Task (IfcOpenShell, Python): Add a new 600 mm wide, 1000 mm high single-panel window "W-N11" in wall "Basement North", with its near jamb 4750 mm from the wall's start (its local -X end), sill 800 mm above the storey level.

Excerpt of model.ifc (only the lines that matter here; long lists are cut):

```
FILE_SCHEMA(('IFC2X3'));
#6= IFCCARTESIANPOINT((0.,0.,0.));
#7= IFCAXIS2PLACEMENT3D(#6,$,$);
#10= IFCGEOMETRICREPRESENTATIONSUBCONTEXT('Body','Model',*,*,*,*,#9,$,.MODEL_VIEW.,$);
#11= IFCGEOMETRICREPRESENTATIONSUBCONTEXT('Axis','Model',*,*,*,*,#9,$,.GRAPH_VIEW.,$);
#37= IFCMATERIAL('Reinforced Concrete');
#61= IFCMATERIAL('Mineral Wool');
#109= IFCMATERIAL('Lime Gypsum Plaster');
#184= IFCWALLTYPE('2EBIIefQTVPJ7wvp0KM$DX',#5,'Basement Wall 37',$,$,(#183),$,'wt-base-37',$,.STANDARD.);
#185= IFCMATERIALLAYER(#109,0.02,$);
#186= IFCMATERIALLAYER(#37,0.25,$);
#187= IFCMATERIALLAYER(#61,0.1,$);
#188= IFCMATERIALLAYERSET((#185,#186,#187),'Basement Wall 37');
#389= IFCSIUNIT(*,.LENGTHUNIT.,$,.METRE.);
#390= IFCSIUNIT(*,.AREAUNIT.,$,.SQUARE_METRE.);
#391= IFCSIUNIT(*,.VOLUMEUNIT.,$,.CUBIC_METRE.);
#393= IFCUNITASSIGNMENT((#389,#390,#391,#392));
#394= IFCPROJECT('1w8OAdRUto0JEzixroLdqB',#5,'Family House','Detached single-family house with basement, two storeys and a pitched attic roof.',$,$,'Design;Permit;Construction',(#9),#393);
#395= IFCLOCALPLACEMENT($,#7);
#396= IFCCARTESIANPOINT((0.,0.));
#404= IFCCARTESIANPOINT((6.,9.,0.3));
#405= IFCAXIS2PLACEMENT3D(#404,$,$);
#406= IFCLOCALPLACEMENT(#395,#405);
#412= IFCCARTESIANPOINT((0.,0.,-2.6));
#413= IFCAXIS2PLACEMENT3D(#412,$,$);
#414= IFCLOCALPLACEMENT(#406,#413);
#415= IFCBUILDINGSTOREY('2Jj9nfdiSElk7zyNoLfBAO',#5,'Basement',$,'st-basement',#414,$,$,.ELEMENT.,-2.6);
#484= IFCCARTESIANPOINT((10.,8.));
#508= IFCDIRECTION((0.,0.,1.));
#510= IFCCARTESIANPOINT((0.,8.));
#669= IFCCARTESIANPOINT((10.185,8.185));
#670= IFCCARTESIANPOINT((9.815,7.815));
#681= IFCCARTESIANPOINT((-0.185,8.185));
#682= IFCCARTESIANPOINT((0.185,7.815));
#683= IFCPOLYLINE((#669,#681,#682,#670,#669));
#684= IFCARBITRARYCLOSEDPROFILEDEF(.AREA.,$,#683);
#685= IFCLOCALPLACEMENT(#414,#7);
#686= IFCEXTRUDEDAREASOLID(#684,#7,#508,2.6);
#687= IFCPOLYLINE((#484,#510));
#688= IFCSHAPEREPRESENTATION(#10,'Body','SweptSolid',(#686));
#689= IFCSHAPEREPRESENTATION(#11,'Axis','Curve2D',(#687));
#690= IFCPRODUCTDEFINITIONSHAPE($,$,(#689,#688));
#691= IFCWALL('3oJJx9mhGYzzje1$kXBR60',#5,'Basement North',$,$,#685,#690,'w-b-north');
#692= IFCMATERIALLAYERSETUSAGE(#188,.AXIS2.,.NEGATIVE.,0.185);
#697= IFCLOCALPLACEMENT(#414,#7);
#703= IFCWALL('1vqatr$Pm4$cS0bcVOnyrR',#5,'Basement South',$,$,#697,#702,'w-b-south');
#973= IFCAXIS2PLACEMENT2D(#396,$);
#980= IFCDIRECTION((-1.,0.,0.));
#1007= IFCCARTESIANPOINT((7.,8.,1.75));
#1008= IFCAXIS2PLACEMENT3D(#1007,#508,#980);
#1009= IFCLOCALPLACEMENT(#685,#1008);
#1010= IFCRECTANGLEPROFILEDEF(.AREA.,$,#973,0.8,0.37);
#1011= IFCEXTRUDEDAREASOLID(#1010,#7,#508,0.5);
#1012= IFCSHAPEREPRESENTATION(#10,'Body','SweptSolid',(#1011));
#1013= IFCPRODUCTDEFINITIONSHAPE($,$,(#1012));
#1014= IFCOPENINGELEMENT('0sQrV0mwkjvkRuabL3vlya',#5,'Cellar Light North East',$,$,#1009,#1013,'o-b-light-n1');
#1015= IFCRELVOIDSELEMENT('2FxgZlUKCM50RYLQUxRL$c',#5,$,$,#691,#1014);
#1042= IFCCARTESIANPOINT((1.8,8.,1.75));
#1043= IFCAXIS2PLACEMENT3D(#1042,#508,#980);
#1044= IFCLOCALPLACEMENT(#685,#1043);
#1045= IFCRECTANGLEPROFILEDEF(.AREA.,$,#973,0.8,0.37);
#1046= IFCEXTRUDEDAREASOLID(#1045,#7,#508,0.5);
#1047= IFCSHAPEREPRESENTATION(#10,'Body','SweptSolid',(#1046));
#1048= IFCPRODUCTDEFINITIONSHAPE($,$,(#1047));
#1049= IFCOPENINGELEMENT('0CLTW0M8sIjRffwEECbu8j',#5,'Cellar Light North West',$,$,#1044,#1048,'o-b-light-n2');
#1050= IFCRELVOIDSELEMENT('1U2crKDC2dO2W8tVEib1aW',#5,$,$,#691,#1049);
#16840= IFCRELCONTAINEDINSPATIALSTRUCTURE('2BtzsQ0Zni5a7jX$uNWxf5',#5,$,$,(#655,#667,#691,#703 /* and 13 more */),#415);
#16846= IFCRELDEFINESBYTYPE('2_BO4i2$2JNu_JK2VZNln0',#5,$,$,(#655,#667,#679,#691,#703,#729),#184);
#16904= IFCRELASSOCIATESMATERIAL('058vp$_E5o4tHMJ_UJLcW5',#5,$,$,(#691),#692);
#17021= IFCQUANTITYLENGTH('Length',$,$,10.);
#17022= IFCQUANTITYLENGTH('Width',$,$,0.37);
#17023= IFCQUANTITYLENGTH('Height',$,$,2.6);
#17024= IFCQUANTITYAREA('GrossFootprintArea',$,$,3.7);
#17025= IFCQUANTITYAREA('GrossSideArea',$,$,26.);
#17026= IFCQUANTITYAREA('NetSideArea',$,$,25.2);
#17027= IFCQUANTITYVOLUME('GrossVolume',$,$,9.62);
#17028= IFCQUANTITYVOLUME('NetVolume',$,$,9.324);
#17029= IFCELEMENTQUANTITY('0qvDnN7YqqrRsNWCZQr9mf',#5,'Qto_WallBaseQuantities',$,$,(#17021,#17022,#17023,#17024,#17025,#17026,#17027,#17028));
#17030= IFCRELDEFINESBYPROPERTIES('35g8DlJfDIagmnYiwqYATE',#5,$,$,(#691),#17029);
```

```python
import numpy as np
import ifcopenshell
import ifcopenshell.api.feature
import ifcopenshell.api.geometry
import ifcopenshell.api.pset
import ifcopenshell.api.root
import ifcopenshell.api.spatial
import ifcopenshell.api.type
import ifcopenshell.geom
import ifcopenshell.util.element
import ifcopenshell.util.placement
import ifcopenshell.util.representation
import ifcopenshell.util.shape
import ifcopenshell.util.unit

model = ifcopenshell.open("model.ifc")
unit_scale = ifcopenshell.util.unit.calculate_unit_scale(model)
area_scale = ifcopenshell.util.unit.calculate_unit_scale(model, "AREAUNIT")
volume_scale = ifcopenshell.util.unit.calculate_unit_scale(model, "VOLUMEUNIT")
settings = ifcopenshell.geom.settings()


def volume(element):
    """Net volume in cubic metres, openings subtracted."""
    shape = ifcopenshell.geom.create_shape(settings, element)
    return ifcopenshell.util.shape.get_volume(shape.geometry)


wall = model.by_guid("3oJJx9mhGYzzje1$kXBR60")
storey = ifcopenshell.util.element.get_container(wall, ifc_class="IfcBuildingStorey")
context = ifcopenshell.util.representation.get_context(model, "Model", "Body", "MODEL_VIEW")
before = volume(wall)

width, height, from_end, sill = 0.6, 1, 4.75, 0.8  # metres

# The wall runs along its own X axis, and the end named is its -X end.
wall_shape = ifcopenshell.geom.create_shape(settings, wall)
x, y, z = ifcopenshell.util.shape.get_vertices(wall_shape.geometry).T
start = x.min() + from_end
face, thickness = float(y.min()), float(y.max() - y.min())
wall_matrix = ifcopenshell.util.placement.get_local_placement(wall.ObjectPlacement)
level = ifcopenshell.util.placement.get_local_placement(storey.ObjectPlacement)[2, 3]


def in_wall(x, y):
    """Placement at x, y metres in the wall's axes, at sill height."""
    matrix = wall_matrix.copy()
    matrix[:, 3] = wall_matrix @ np.array([x / unit_scale, y / unit_scale, 0.0, 1.0])
    matrix[2, 3] = level + sill / unit_scale
    return matrix


# Opening: a box that overshoots both wall faces by 50 mm.
opening = ifcopenshell.api.root.create_entity(model, ifc_class="IfcOpeningElement")
box = ifcopenshell.api.geometry.add_wall_representation(
    model, context=context, length=width, height=height, thickness=thickness + 0.1
)
ifcopenshell.api.geometry.assign_representation(model, product=opening, representation=box)
ifcopenshell.api.geometry.edit_object_placement(model, product=opening, matrix=in_wall(start, face - 0.05), is_si=False)
ifcopenshell.api.feature.add_feature(model, feature=opening, element=wall)

window = ifcopenshell.api.root.create_entity(model, ifc_class="IfcWindow", name="W-N11")
window.OverallWidth, window.OverallHeight = width / unit_scale, height / unit_scale
body = ifcopenshell.api.geometry.add_window_representation(
    model,
    context=context,
    overall_width=window.OverallWidth,
    overall_height=window.OverallHeight,
    partition_type="SINGLE_PANEL",
)
ifcopenshell.api.geometry.assign_representation(model, product=window, representation=body)
ifcopenshell.api.spatial.assign_container(model, products=[window], relating_structure=storey)
fills = ifcopenshell.api.feature.add_filling(model, opening=opening, element=window)
fills.OwnerHistory = window.OwnerHistory  # required in IFC2X3

# IFC2X3 keeps the operation on the window style.
style = ifcopenshell.api.root.create_entity(model, ifc_class="IfcWindowStyle", name="W-N11")
style.OperationType, style.ConstructionType = "SINGLE_PANEL", "NOTDEFINED"
style.ParameterTakesPrecedence = style.Sizeable = False
ifcopenshell.api.type.assign_type(model, related_objects=[window], relating_type=style)

# Centre the window in the wall's thickness.
ifcopenshell.api.geometry.edit_object_placement(model, product=window, matrix=in_wall(start, face), is_si=False)
window_shape = ifcopenshell.geom.create_shape(settings, window)
depth = ifcopenshell.util.shape.get_vertices(window_shape.geometry)[:, 1]
offset = face + thickness / 2 - (depth.min() + depth.max()) / 2
ifcopenshell.api.geometry.edit_object_placement(model, product=window, matrix=in_wall(start, offset), is_si=False)

after = volume(wall)

# Update the wall's stored quantities.
qto = model.by_id(ifcopenshell.util.element.get_pset(wall, "Qto_WallBaseQuantities", should_inherit=False)["id"])
ifcopenshell.api.pset.edit_qto(model, qto=qto, properties={
    "NetSideArea": after / thickness / area_scale,
    "NetVolume": after / volume_scale,
})

print(f"wall volume {before:.3f} -> {after:.3f} m3")

model.write("model-out.ifc")
```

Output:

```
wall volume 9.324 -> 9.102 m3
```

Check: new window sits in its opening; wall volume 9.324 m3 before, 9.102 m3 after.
